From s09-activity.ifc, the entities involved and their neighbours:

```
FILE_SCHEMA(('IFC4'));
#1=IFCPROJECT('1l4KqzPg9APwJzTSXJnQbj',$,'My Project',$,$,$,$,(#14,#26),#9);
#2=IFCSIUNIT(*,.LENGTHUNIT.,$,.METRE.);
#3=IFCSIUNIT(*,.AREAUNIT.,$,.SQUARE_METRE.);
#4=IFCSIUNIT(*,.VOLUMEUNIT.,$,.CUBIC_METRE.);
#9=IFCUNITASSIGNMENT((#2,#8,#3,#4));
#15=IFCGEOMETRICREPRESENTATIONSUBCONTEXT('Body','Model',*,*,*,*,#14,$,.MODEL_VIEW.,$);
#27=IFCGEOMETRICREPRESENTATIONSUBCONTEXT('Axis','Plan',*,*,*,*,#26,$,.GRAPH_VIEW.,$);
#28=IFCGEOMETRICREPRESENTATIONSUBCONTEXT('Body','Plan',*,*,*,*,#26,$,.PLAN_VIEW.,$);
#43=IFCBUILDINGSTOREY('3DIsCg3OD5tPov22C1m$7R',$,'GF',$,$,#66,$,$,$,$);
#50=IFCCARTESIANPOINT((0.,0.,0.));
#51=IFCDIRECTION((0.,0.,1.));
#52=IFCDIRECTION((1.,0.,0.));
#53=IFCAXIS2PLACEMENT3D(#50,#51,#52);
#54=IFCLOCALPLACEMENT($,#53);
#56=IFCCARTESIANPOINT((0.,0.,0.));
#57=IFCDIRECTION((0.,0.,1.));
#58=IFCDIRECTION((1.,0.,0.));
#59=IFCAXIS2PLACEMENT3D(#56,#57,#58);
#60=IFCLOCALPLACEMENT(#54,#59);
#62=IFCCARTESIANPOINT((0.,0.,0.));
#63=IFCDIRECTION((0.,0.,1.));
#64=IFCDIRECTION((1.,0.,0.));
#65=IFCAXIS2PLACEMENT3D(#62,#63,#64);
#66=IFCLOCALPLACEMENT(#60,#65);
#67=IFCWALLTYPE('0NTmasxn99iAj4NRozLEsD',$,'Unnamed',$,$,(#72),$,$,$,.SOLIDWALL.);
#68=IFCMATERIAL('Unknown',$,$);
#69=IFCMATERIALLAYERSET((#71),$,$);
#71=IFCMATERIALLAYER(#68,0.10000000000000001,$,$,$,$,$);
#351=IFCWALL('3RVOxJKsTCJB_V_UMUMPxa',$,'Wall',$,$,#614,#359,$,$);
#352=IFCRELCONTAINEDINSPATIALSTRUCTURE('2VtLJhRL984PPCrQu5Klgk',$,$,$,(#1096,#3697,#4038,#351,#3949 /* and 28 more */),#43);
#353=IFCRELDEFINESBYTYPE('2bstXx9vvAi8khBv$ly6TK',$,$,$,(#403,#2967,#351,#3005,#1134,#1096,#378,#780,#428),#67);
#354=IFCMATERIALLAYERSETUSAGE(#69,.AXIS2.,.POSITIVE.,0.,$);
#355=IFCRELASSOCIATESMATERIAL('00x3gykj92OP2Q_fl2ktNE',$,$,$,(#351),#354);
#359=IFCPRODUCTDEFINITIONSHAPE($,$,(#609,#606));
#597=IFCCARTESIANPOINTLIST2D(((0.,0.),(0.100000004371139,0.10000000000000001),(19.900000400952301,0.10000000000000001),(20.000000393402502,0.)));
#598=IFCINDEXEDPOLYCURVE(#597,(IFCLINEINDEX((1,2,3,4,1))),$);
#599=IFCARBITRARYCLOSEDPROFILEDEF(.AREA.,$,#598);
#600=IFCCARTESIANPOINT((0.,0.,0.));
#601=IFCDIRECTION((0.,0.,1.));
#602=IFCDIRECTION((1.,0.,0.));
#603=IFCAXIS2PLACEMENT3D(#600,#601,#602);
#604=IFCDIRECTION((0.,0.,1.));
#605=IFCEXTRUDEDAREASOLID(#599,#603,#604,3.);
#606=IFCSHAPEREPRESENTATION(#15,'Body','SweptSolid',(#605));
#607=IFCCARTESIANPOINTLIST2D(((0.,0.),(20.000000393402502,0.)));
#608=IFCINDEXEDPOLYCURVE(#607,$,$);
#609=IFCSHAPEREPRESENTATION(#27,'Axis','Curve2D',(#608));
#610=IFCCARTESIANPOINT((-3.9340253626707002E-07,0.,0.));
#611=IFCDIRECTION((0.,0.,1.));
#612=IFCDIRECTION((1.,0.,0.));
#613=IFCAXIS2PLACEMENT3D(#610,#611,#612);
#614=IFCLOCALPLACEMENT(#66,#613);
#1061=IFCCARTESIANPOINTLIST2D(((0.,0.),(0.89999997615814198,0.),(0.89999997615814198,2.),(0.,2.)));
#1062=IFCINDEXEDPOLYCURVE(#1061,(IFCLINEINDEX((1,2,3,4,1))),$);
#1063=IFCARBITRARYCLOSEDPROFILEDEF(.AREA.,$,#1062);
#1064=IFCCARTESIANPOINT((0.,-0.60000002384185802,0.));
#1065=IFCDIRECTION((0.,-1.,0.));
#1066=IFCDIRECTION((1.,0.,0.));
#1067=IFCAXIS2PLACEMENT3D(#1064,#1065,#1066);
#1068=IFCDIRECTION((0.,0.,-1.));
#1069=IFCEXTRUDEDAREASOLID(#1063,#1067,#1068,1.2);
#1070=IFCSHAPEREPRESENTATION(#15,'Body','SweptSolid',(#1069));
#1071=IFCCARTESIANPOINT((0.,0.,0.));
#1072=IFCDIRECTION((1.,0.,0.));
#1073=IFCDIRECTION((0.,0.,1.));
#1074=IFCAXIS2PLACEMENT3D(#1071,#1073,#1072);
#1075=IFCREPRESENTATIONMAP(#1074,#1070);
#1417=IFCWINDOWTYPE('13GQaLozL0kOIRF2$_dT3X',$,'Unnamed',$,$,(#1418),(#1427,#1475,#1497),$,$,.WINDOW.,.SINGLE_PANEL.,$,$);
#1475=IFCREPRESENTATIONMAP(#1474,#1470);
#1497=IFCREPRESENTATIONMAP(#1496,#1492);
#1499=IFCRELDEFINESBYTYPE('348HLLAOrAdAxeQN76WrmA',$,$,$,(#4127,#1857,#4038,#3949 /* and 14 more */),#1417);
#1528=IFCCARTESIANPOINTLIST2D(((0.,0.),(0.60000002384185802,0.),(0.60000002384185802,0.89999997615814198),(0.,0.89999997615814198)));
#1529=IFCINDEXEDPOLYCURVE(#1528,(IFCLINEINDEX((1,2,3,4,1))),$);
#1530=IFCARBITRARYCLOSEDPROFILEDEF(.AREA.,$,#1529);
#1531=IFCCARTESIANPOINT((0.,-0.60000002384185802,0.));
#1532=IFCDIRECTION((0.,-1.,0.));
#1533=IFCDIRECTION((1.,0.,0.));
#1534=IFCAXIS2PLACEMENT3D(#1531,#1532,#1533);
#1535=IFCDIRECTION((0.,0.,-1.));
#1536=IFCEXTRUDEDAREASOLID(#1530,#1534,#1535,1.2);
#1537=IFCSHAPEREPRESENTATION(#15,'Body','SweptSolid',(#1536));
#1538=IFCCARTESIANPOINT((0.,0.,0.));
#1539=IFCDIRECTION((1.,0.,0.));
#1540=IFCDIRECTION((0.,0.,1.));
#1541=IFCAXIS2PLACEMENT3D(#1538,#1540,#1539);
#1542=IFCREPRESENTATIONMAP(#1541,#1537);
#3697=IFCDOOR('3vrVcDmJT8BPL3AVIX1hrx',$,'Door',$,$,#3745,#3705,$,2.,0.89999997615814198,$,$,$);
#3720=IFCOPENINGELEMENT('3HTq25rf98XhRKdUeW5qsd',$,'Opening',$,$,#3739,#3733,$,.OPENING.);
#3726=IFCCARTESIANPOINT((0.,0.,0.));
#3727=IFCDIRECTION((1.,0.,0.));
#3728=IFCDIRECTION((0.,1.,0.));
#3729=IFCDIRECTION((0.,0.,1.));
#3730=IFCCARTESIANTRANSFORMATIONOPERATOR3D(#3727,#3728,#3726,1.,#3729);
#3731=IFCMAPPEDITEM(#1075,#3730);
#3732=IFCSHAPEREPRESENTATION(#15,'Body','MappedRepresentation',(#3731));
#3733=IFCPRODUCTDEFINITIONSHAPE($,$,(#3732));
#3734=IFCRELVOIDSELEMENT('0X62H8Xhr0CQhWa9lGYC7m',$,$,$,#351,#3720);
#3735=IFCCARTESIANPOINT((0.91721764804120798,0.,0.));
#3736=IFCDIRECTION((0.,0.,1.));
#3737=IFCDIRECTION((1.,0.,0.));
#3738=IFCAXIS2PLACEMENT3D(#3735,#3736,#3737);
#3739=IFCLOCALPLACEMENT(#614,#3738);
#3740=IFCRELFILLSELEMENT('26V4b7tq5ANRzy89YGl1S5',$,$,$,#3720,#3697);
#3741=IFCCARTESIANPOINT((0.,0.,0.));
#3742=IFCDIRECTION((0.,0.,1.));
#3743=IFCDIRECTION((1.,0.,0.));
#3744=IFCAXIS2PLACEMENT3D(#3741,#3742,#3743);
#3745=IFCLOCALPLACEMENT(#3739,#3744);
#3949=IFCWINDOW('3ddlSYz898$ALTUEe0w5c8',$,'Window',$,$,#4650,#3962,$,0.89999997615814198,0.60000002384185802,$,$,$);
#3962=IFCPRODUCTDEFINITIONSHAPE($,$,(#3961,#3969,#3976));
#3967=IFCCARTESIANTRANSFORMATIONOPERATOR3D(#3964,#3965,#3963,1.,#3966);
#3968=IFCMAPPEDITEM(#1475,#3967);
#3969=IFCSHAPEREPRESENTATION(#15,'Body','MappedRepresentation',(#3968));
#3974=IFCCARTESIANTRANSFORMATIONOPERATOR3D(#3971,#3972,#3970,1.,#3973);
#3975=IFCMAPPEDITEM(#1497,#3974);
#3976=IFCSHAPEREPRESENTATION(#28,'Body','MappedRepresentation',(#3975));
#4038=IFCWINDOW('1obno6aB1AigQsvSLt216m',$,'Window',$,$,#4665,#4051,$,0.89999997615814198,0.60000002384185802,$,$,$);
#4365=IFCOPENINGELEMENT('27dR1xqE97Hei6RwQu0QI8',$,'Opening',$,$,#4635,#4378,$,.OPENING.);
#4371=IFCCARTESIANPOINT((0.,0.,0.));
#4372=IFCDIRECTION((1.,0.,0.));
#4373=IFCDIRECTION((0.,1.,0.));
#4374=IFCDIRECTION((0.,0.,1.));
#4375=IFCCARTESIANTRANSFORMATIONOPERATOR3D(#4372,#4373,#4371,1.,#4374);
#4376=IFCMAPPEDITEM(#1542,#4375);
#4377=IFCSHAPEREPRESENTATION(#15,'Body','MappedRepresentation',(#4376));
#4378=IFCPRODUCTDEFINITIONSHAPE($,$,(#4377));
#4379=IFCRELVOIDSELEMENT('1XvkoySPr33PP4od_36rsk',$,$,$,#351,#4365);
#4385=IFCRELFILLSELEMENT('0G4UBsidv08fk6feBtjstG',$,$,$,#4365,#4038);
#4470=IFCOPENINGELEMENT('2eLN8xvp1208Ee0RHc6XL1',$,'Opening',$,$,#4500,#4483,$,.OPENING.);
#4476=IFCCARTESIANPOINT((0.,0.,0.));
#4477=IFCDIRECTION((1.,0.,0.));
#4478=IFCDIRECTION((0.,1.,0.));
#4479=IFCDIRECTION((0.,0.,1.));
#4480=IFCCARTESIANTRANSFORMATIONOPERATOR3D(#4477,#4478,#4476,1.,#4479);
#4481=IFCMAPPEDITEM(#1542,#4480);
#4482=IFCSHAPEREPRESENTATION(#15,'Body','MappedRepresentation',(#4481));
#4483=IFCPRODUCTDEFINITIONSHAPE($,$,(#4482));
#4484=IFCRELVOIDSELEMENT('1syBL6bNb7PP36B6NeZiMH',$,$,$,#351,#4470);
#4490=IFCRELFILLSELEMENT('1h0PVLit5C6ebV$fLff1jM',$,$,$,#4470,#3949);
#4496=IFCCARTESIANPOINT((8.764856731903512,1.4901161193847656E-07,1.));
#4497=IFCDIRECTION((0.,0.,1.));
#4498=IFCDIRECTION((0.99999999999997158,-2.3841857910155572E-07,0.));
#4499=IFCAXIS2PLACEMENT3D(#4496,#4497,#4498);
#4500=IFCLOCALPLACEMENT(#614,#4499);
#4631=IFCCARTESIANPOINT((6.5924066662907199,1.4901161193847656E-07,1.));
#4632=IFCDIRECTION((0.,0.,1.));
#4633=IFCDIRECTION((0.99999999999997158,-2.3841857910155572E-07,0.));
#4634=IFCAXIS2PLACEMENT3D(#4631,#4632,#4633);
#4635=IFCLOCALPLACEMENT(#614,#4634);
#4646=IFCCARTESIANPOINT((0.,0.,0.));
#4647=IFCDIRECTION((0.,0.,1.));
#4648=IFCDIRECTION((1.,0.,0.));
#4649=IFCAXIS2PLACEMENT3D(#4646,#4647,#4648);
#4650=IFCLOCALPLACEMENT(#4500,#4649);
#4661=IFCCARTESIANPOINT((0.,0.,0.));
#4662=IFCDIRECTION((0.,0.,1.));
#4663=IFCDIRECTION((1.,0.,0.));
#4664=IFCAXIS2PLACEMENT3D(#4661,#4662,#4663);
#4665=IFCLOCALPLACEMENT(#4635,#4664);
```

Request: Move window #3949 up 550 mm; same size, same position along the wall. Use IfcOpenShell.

```python
import numpy as np
import ifcopenshell
import ifcopenshell.api.geometry
import ifcopenshell.util.placement
import ifcopenshell.util.unit

model = ifcopenshell.open("s09-activity.ifc")
unit_scale = ifcopenshell.util.unit.calculate_unit_scale(model)

window = model.by_id(3949)
opening = window.FillsVoids[0].RelatingOpeningElement
dz = 0.55

shift = np.array([0.0, 0.0, dz])
# The window is placed relative to its opening, so it follows when the opening moves.
matrix = ifcopenshell.util.placement.get_local_placement(opening.ObjectPlacement)
matrix[:3, 3] += shift
ifcopenshell.api.geometry.edit_object_placement(
    model, product=opening, matrix=matrix, is_si=False, should_transform_children=True
)

print(f"moved by {dz * unit_scale:+.3f} m")

model.write("s09-activity_updated.ifc")
```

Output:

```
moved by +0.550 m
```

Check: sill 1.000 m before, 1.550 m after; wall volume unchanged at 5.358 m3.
